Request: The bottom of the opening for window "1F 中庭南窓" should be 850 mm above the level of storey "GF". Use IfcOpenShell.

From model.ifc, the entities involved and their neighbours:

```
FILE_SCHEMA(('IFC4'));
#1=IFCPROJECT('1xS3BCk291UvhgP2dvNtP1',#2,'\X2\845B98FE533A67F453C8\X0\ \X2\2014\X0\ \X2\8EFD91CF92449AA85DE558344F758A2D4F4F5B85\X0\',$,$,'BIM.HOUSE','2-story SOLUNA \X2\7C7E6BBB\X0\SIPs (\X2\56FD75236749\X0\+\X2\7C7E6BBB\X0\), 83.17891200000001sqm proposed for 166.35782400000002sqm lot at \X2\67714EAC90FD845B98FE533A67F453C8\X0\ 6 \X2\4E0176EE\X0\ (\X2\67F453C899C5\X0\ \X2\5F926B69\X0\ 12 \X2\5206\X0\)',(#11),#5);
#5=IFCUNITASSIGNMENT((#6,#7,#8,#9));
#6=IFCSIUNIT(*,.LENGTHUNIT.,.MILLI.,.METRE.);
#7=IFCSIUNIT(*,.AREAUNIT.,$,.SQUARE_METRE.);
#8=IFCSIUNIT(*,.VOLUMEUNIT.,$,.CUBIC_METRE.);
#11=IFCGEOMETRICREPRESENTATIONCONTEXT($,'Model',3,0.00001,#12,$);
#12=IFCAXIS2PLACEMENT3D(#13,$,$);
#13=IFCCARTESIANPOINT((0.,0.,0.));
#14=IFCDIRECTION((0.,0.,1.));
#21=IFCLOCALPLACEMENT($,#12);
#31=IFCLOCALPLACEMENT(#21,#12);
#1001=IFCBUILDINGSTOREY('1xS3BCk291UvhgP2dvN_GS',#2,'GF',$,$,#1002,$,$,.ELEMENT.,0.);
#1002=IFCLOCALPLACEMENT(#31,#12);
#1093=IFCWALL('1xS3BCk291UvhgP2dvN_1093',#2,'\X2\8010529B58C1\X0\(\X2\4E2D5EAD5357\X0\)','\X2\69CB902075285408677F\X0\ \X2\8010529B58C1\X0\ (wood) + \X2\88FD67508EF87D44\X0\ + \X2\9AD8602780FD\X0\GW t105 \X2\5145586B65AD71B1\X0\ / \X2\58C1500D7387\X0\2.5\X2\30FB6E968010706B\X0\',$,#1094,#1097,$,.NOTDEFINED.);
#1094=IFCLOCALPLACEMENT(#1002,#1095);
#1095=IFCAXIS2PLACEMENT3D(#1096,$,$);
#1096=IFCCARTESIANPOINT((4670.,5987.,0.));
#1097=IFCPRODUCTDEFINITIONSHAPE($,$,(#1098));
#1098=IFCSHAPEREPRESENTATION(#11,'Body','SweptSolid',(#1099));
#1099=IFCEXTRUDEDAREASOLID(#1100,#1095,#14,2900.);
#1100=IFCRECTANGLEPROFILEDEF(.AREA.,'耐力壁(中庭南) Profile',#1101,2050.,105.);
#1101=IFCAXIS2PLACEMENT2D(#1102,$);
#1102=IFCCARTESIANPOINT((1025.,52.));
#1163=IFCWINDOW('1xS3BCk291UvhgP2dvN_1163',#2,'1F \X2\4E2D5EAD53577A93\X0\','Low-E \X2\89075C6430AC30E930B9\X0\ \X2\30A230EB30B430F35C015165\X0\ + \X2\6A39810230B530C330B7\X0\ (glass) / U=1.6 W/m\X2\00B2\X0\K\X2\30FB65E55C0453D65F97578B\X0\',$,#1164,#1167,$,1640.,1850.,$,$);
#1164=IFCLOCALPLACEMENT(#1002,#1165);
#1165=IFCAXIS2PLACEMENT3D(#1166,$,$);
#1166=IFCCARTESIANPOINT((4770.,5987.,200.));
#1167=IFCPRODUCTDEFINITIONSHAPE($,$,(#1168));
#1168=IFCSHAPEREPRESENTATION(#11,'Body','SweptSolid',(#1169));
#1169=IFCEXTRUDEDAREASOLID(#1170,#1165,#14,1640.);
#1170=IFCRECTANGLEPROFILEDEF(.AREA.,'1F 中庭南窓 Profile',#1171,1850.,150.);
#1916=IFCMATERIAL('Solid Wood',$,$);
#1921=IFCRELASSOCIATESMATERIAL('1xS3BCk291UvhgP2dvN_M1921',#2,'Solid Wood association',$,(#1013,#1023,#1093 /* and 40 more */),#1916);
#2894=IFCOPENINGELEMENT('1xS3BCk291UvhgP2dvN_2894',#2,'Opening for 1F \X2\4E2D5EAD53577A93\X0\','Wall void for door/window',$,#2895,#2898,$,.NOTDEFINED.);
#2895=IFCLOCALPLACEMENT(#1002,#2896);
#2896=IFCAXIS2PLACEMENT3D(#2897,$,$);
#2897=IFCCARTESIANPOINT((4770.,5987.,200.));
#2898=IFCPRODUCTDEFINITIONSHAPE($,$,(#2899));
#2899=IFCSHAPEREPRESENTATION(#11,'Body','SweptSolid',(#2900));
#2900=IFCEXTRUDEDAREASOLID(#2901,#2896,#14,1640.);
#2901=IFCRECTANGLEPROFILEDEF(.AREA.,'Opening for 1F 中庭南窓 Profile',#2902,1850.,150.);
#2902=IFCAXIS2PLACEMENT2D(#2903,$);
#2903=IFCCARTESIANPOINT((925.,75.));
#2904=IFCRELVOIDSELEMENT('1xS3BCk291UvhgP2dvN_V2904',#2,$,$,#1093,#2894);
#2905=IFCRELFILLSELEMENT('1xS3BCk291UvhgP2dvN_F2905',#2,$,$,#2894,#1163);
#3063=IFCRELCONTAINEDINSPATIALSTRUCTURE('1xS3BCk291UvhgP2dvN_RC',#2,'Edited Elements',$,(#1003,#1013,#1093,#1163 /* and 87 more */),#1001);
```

```python
import numpy as np
import ifcopenshell
import ifcopenshell.api.geometry
import ifcopenshell.geom
import ifcopenshell.util.element
import ifcopenshell.util.placement
import ifcopenshell.util.shape
import ifcopenshell.util.unit

model = ifcopenshell.open("model.ifc")
unit_scale = ifcopenshell.util.unit.calculate_unit_scale(model)

window = model.by_id(1163)
opening = window.FillsVoids[0].RelatingOpeningElement
storey = ifcopenshell.util.element.get_container(window, ifc_class="IfcBuildingStorey")
level = ifcopenshell.util.placement.get_local_placement(storey.ObjectPlacement)[2, 3]

# The opening's origin need not be at the sill, so measure its lowest point.
shape = ifcopenshell.geom.create_shape(ifcopenshell.geom.settings(), opening)
bottom = ifcopenshell.util.shape.get_shape_bottom_elevation(shape, shape.geometry) / unit_scale
dz = level + 0.85 / unit_scale - bottom

shift = np.array([0.0, 0.0, dz])
# The window is not placed relative to its opening, so move both.
for product in (opening, window):
    matrix = ifcopenshell.util.placement.get_local_placement(product.ObjectPlacement)
    matrix[:3, 3] += shift
    ifcopenshell.api.geometry.edit_object_placement(model, product=product, matrix=matrix, is_si=False)

print(f"moved by {dz * unit_scale:+.3f} m")

model.write("model_updated.ifc")
```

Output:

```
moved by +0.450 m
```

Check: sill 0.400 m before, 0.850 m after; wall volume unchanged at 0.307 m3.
